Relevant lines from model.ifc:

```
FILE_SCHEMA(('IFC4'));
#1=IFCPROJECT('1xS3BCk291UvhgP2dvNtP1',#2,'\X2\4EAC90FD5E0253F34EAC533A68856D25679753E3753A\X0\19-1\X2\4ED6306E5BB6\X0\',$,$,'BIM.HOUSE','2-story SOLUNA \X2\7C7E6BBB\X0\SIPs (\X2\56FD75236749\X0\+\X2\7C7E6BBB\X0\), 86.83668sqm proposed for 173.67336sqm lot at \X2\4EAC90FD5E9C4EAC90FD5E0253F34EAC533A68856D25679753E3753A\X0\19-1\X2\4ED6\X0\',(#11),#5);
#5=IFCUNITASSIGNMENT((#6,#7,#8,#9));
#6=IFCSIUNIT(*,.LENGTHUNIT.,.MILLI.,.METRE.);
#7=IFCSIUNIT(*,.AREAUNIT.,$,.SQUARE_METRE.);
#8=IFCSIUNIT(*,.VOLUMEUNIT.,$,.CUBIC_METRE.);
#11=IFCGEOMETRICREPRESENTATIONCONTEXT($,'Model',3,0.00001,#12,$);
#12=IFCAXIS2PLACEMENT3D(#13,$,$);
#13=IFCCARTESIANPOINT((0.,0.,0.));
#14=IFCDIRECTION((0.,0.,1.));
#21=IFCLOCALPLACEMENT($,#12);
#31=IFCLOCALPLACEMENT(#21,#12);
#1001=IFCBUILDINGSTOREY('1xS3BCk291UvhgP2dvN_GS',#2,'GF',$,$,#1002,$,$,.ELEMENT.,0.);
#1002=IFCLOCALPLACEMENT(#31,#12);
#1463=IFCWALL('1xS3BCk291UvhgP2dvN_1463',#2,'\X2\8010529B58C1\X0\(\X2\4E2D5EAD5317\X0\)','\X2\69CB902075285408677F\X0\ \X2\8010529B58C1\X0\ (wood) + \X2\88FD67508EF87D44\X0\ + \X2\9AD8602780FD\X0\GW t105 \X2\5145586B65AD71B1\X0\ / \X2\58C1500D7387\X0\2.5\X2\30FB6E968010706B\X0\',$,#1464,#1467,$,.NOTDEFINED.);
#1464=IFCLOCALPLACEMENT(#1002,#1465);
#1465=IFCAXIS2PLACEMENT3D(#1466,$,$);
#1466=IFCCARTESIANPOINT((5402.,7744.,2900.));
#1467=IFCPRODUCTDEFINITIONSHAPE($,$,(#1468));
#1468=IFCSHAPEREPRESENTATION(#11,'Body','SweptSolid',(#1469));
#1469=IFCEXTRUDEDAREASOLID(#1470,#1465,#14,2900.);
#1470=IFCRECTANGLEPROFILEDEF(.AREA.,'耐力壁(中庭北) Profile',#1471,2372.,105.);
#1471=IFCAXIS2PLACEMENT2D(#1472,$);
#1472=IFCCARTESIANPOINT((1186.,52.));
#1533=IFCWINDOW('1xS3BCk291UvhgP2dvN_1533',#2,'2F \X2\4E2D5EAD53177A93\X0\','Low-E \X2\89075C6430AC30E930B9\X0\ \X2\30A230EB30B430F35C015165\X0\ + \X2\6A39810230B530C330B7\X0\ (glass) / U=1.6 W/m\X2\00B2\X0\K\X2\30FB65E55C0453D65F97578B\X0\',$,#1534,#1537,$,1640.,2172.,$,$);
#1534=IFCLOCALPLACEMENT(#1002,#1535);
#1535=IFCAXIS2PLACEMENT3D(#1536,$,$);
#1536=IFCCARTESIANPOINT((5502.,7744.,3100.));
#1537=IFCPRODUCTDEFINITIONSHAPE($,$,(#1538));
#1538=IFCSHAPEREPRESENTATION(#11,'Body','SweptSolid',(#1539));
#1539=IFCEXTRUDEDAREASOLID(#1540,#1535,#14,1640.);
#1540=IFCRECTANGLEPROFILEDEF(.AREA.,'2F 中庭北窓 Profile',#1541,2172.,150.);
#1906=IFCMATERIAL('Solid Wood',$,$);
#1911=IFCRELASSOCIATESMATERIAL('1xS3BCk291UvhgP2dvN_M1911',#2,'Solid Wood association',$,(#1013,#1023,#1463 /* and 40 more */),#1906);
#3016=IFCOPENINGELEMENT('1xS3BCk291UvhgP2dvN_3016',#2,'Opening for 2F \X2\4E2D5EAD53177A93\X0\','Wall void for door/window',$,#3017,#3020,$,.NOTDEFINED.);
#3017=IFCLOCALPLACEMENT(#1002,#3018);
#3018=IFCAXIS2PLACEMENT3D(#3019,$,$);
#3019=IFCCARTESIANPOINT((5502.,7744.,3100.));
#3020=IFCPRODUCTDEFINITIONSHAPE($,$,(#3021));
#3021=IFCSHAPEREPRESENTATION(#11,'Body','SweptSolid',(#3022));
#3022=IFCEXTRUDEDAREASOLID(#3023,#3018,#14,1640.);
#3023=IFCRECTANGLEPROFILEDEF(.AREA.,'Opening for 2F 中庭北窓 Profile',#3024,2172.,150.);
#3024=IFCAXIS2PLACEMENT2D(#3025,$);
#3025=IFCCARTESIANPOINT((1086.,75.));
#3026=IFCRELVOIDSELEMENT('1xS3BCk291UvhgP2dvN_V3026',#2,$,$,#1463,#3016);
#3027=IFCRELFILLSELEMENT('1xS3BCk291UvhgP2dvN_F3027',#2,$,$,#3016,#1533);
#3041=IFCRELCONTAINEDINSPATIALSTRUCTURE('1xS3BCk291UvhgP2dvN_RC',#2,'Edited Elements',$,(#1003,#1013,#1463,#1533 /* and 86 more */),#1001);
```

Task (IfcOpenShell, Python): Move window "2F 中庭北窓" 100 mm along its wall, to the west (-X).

```python
import ifcopenshell
import ifcopenshell.api.geometry
import ifcopenshell.util.placement

model = ifcopenshell.open("model.ifc")

window = model.by_guid("1xS3BCk291UvhgP2dvN_1533")
opening = window.FillsVoids[0].RelatingOpeningElement
wall = opening.VoidsElements[0].RelatingBuildingElement

wall_matrix = ifcopenshell.util.placement.get_local_placement(wall.ObjectPlacement)
shift = wall_matrix[:3, 0] * -100.0
before = ifcopenshell.util.placement.get_local_placement(window.ObjectPlacement)[:3, 3].copy()

# The window is not placed relative to its opening, so move both.
for product in (opening, window):
    matrix = ifcopenshell.util.placement.get_local_placement(product.ObjectPlacement)
    matrix[:3, 3] += shift
    ifcopenshell.api.geometry.edit_object_placement(model, product=product, matrix=matrix, is_si=False)

after = ifcopenshell.util.placement.get_local_placement(window.ObjectPlacement)[:3, 3]
print("window moved by", (after - before).round(3) + 0.0)

model.write("model-out.ifc")
```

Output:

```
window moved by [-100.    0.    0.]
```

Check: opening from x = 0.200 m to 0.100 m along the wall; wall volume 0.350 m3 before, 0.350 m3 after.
